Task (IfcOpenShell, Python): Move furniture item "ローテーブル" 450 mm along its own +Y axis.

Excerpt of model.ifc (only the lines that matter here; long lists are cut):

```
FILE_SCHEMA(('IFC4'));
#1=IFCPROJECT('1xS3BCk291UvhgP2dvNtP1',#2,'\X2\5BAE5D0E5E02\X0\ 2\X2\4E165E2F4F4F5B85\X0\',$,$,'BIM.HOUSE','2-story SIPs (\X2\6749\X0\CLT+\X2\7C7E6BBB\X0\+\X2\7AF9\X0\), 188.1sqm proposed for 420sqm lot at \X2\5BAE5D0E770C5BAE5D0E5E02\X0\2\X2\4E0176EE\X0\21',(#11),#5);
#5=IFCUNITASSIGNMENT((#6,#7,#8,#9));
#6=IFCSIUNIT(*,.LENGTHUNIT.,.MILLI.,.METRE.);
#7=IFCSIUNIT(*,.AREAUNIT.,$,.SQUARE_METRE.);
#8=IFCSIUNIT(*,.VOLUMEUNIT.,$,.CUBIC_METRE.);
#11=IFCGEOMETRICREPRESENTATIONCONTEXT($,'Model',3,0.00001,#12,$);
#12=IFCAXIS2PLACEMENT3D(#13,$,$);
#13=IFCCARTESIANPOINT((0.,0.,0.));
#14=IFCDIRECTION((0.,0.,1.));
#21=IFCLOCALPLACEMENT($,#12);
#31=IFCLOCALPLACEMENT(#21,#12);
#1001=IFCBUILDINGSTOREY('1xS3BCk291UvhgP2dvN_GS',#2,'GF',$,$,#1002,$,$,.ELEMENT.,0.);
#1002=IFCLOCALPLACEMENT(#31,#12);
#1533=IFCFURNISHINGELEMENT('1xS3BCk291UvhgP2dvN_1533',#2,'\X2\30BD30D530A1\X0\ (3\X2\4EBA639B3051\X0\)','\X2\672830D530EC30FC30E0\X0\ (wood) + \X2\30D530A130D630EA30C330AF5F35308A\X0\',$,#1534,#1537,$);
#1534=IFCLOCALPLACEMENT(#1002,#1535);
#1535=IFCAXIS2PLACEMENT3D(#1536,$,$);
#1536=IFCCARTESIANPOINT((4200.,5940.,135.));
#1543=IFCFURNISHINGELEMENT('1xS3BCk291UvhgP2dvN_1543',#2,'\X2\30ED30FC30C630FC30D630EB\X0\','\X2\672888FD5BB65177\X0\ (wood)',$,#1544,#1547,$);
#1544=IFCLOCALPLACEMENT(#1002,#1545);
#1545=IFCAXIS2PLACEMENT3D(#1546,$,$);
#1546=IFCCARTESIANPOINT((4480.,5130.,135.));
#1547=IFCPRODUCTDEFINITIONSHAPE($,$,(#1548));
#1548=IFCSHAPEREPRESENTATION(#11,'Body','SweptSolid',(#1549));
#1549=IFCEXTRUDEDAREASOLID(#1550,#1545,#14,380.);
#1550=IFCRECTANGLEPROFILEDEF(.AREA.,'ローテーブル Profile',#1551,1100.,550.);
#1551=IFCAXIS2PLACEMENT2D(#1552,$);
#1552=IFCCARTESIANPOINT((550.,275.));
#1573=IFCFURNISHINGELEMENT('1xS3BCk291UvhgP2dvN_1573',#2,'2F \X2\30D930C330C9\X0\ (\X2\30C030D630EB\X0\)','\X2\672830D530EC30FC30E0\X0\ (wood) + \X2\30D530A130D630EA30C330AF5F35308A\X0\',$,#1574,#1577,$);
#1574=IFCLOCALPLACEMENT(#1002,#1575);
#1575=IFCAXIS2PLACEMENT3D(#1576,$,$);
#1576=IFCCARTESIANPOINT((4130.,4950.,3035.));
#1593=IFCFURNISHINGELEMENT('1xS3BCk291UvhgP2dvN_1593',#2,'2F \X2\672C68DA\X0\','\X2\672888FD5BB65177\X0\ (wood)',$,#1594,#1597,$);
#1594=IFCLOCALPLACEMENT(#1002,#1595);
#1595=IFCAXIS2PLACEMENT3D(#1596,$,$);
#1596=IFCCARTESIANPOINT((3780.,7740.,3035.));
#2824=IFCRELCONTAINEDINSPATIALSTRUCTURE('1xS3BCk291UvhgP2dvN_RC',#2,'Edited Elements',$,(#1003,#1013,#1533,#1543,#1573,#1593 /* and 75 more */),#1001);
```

```python
import ifcopenshell
import ifcopenshell.api.geometry
import ifcopenshell.util.placement
import ifcopenshell.util.unit

model = ifcopenshell.open("model.ifc")
unit_scale = ifcopenshell.util.unit.calculate_unit_scale(model)

item = model.by_guid("1xS3BCk291UvhgP2dvN_1543")
matrix = ifcopenshell.util.placement.get_local_placement(item.ObjectPlacement)
matrix[:3, 3] += matrix[:3, 1] * 0.45 / unit_scale
ifcopenshell.api.geometry.edit_object_placement(model, product=item, matrix=matrix, is_si=False)

print(ifcopenshell.util.placement.get_local_placement(item.ObjectPlacement).round(3) + 0.0)

model.write("model_updated.ifc")
```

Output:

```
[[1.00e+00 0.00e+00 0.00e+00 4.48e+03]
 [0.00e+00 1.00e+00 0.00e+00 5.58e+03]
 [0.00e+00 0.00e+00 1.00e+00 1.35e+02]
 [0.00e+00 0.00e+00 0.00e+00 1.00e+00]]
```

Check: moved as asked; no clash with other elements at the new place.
